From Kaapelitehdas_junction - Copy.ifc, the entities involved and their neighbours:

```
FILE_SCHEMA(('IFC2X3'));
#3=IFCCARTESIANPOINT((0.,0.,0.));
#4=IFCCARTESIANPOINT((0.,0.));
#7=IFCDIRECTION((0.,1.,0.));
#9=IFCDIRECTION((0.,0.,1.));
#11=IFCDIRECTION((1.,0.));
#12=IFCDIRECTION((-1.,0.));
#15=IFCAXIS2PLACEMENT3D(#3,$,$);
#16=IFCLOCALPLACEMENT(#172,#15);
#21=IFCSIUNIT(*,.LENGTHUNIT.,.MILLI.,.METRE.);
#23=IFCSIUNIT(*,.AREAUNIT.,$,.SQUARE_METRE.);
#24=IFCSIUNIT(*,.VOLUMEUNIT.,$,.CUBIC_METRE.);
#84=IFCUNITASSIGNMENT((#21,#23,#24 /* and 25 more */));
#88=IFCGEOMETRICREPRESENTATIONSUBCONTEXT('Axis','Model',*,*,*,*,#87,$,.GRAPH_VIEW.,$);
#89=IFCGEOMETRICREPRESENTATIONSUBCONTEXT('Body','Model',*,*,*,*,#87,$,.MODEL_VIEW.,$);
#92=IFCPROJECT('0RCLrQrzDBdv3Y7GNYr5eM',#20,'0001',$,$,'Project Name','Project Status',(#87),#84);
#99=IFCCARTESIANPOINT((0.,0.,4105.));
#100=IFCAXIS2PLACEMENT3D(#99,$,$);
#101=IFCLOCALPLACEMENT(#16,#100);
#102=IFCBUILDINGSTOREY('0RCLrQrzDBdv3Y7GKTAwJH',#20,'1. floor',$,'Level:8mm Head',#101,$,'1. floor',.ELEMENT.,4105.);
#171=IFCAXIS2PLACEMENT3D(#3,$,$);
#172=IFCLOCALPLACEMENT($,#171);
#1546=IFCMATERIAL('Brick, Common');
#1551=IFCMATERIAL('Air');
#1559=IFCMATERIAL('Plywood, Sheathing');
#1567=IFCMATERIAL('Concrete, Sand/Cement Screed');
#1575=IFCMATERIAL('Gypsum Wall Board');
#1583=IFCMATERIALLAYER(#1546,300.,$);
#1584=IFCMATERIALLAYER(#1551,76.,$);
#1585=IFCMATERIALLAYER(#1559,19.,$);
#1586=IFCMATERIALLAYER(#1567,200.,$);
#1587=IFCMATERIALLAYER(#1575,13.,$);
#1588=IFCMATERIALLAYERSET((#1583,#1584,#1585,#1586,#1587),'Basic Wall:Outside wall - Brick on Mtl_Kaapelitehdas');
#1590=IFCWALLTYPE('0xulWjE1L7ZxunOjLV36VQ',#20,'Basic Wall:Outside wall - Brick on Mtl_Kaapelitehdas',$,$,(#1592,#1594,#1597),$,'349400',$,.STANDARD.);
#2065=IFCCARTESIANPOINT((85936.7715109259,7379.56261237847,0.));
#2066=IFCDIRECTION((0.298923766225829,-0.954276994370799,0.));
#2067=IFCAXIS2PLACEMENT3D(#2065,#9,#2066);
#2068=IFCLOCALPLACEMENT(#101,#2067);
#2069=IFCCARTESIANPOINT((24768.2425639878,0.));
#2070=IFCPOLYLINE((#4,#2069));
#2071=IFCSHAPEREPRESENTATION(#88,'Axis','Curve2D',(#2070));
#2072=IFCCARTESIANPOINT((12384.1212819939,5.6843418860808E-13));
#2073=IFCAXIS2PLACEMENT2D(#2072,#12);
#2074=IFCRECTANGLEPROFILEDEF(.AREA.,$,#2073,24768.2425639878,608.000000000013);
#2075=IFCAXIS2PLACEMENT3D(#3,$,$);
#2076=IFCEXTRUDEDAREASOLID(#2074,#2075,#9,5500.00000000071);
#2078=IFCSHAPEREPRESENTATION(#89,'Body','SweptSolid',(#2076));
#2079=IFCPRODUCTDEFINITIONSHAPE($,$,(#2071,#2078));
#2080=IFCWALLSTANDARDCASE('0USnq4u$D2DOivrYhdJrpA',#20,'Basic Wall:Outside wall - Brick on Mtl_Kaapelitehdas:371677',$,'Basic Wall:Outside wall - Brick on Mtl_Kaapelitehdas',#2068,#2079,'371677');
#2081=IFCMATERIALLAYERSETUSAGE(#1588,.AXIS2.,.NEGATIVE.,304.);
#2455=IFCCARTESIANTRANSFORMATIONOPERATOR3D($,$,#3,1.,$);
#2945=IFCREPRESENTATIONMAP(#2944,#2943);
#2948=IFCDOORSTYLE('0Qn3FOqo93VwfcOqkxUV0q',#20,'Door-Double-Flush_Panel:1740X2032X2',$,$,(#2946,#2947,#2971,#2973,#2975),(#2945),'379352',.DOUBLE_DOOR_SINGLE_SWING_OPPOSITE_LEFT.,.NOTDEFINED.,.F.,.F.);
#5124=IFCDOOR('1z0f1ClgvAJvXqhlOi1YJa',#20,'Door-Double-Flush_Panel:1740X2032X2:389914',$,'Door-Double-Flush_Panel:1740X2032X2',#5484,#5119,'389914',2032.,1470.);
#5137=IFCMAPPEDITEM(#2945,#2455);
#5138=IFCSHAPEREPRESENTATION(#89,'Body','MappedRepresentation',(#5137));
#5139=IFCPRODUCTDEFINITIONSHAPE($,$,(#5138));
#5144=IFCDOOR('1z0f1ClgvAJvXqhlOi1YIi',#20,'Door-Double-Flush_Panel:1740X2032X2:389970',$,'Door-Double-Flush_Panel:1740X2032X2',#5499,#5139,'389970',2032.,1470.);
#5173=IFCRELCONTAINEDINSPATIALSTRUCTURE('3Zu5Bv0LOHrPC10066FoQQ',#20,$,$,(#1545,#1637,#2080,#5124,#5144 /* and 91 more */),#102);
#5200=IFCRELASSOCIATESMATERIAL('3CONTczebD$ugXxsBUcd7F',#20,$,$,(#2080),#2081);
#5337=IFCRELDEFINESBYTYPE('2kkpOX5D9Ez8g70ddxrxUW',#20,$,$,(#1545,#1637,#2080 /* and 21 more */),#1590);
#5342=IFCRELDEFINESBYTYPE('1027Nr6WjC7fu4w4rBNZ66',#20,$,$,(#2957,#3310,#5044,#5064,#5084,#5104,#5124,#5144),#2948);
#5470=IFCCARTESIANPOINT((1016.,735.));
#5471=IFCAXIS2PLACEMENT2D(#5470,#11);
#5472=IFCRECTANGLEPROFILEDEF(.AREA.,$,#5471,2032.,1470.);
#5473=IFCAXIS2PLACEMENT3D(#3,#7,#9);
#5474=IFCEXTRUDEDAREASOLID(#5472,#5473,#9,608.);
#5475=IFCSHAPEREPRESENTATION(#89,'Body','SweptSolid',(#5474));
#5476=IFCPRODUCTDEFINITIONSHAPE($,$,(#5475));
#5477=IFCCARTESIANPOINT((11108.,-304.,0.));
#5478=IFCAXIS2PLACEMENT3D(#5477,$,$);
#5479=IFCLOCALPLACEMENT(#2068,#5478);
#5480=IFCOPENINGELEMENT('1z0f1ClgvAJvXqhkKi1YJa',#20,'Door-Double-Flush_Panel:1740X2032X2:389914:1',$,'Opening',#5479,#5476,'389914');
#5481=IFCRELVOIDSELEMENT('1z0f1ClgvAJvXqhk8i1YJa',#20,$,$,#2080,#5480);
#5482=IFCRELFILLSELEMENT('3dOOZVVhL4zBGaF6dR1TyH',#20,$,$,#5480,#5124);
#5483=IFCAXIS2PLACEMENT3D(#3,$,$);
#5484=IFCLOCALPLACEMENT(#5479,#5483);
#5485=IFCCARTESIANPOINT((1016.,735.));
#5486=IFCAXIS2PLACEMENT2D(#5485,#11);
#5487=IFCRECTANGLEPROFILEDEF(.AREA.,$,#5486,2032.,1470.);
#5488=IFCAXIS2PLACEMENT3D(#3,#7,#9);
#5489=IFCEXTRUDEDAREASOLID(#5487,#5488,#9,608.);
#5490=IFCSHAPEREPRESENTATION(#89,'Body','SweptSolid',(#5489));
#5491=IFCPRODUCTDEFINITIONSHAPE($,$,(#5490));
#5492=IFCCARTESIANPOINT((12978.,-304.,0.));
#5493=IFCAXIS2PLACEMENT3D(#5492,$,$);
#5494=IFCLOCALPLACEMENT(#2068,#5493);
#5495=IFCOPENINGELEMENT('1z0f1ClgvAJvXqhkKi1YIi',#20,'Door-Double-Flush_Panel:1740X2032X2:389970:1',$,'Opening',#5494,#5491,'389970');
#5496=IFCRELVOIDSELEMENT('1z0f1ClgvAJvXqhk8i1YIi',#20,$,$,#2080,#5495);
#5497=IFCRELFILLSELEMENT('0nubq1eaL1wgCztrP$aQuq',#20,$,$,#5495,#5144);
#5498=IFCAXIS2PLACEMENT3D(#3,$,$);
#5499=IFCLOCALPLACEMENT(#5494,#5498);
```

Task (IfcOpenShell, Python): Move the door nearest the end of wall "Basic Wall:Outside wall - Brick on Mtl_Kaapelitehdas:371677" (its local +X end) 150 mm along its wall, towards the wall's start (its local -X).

```python
import ifcopenshell
import ifcopenshell.api.geometry
import ifcopenshell.util.placement

model = ifcopenshell.open("Kaapelitehdas_junction - Copy.ifc")

door = model.by_id(5144)
opening = door.FillsVoids[0].RelatingOpeningElement
wall = opening.VoidsElements[0].RelatingBuildingElement

wall_matrix = ifcopenshell.util.placement.get_local_placement(wall.ObjectPlacement)
shift = wall_matrix[:3, 0] * -150.0
before = ifcopenshell.util.placement.get_local_placement(door.ObjectPlacement)[:3, 3].copy()

# The door is placed relative to its opening, so it follows when the opening moves.
matrix = ifcopenshell.util.placement.get_local_placement(opening.ObjectPlacement)
matrix[:3, 3] += shift
ifcopenshell.api.geometry.edit_object_placement(
    model, product=opening, matrix=matrix, is_si=False, should_transform_children=True
)

after = ifcopenshell.util.placement.get_local_placement(door.ObjectPlacement)[:3, 3]
print("door moved by", (after - before).round(3) + 0.0)

model.write("Kaapelitehdas_junction - Copy_v2.ifc")
```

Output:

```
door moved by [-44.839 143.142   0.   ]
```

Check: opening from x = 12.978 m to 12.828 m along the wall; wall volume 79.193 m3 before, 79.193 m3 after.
